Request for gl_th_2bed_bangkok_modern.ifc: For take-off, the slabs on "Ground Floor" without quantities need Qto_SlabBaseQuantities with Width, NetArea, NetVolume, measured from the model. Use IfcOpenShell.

First a look at what the model holds.

```python
import ifcopenshell
import ifcopenshell.util.element
import ifcopenshell.util.unit

model = ifcopenshell.open("gl_th_2bed_bangkok_modern.ifc")
print(model.schema)
for unit_type in ("LENGTHUNIT", "AREAUNIT", "VOLUMEUNIT"):
    print(unit_type, ifcopenshell.util.unit.calculate_unit_scale(model, unit_type))
storey = next(s for s in model.by_type("IfcBuildingStorey") if s.Name == "Ground Floor")
slabs = [e for e in ifcopenshell.util.element.get_decomposition(storey) if e.is_a("IfcSlab")]
for e in sorted(slabs, key=lambda e: e.id()):
    print(e.id(), e.is_a(), e.Name, list(ifcopenshell.util.element.get_psets(e, qtos_only=True)), sep=" | ")
```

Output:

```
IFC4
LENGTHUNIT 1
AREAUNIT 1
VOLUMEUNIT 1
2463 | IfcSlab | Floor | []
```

```python
import ifcopenshell
import ifcopenshell.api.pset
import ifcopenshell.geom
import ifcopenshell.util.element
import ifcopenshell.util.shape
import ifcopenshell.util.unit

model = ifcopenshell.open("gl_th_2bed_bangkok_modern.ifc")
unit_scale = ifcopenshell.util.unit.calculate_unit_scale(model)
area_scale = ifcopenshell.util.unit.calculate_unit_scale(model, "AREAUNIT")
volume_scale = ifcopenshell.util.unit.calculate_unit_scale(model, "VOLUMEUNIT")
settings = ifcopenshell.geom.settings()

storey = next(s for s in model.by_type("IfcBuildingStorey") if s.Name == "Ground Floor")
slabs = [e for e in ifcopenshell.util.element.get_decomposition(storey) if e.is_a("IfcSlab")]

for e in sorted(slabs, key=lambda e: e.id()):
    if ifcopenshell.util.element.get_psets(e, qtos_only=True, should_inherit=False):
        continue
    # Geometry comes back in metres, in the element's own axes.
    shape = ifcopenshell.geom.create_shape(settings, e)
    values = {
        "Width": ifcopenshell.util.shape.get_z(shape.geometry) / unit_scale,
        "NetArea": ifcopenshell.util.shape.get_footprint_area(shape.geometry) / area_scale,
        "NetVolume": ifcopenshell.util.shape.get_volume(shape.geometry) / volume_scale,
    }
    qto = ifcopenshell.api.pset.add_qto(model, product=e, name="Qto_SlabBaseQuantities")
    ifcopenshell.api.pset.edit_qto(model, qto=qto, properties=values)
    print(e.id(), {k: round(v, 3) for k, v in values.items()})

model.write("gl_th_2bed_bangkok_modern-out.ifc")
```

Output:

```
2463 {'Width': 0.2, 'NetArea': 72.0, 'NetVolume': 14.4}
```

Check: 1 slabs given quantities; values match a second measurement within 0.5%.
